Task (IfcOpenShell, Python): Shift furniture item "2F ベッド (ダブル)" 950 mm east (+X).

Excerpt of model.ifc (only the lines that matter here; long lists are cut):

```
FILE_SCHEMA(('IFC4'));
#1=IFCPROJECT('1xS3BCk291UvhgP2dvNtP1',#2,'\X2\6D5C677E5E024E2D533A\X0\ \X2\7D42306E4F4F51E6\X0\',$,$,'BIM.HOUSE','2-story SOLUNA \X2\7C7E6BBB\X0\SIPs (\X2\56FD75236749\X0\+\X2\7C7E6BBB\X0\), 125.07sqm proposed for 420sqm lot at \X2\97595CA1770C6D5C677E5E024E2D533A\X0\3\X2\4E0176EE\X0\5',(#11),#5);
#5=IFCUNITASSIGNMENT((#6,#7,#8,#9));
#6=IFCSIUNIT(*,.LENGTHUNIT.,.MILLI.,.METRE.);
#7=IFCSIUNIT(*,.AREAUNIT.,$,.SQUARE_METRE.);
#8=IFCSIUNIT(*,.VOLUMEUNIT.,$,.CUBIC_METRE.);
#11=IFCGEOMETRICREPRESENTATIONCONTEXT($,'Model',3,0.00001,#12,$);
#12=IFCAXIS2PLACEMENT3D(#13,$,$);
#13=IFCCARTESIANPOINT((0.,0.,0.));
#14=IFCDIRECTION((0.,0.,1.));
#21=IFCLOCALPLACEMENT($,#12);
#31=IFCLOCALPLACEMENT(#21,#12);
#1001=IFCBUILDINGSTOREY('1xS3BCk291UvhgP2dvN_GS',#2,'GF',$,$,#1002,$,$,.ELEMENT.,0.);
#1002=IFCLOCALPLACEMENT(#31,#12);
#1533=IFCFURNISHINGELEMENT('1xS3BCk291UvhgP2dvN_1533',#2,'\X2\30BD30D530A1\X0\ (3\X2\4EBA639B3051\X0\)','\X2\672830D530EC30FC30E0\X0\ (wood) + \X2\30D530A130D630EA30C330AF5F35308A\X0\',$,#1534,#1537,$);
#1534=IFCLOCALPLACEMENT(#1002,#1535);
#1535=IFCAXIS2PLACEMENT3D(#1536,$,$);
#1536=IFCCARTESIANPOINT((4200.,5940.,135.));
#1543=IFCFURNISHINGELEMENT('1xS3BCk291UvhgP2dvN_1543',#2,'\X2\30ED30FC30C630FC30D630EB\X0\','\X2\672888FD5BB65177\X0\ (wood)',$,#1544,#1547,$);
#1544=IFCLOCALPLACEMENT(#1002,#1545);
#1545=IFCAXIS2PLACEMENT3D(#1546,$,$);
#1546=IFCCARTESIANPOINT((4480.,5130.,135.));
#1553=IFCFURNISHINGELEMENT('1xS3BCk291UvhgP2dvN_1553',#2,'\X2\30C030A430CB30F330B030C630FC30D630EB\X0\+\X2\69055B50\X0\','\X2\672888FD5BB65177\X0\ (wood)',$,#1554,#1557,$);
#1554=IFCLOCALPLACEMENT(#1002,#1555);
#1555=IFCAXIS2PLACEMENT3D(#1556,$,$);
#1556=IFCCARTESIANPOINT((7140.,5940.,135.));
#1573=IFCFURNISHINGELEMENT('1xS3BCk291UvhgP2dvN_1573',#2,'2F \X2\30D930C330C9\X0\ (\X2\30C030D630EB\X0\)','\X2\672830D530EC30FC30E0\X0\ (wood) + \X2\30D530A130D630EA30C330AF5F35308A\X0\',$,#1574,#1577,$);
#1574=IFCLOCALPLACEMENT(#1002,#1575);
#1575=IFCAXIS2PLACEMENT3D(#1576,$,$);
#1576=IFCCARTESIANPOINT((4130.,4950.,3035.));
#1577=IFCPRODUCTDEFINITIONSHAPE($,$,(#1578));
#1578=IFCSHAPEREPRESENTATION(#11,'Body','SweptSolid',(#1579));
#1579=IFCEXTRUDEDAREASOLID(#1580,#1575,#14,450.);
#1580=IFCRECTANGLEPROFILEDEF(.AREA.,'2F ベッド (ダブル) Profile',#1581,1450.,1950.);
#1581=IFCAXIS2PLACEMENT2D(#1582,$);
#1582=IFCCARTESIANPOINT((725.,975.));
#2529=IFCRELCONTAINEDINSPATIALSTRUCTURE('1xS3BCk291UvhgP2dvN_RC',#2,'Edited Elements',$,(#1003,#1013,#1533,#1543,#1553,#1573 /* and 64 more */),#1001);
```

```python
import ifcopenshell
import ifcopenshell.api.geometry
import ifcopenshell.util.placement

model = ifcopenshell.open("model.ifc")

item = model.by_guid("1xS3BCk291UvhgP2dvN_1573")
matrix = ifcopenshell.util.placement.get_local_placement(item.ObjectPlacement)
matrix[0, 3] += 950.0
ifcopenshell.api.geometry.edit_object_placement(model, product=item, matrix=matrix, is_si=False)

print(ifcopenshell.util.placement.get_local_placement(item.ObjectPlacement).round(3) + 0.0)

model.write("model-out.ifc")
```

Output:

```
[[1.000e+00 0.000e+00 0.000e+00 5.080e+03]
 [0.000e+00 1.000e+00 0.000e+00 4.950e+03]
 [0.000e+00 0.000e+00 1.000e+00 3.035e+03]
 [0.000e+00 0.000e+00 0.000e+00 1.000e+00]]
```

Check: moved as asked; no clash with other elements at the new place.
